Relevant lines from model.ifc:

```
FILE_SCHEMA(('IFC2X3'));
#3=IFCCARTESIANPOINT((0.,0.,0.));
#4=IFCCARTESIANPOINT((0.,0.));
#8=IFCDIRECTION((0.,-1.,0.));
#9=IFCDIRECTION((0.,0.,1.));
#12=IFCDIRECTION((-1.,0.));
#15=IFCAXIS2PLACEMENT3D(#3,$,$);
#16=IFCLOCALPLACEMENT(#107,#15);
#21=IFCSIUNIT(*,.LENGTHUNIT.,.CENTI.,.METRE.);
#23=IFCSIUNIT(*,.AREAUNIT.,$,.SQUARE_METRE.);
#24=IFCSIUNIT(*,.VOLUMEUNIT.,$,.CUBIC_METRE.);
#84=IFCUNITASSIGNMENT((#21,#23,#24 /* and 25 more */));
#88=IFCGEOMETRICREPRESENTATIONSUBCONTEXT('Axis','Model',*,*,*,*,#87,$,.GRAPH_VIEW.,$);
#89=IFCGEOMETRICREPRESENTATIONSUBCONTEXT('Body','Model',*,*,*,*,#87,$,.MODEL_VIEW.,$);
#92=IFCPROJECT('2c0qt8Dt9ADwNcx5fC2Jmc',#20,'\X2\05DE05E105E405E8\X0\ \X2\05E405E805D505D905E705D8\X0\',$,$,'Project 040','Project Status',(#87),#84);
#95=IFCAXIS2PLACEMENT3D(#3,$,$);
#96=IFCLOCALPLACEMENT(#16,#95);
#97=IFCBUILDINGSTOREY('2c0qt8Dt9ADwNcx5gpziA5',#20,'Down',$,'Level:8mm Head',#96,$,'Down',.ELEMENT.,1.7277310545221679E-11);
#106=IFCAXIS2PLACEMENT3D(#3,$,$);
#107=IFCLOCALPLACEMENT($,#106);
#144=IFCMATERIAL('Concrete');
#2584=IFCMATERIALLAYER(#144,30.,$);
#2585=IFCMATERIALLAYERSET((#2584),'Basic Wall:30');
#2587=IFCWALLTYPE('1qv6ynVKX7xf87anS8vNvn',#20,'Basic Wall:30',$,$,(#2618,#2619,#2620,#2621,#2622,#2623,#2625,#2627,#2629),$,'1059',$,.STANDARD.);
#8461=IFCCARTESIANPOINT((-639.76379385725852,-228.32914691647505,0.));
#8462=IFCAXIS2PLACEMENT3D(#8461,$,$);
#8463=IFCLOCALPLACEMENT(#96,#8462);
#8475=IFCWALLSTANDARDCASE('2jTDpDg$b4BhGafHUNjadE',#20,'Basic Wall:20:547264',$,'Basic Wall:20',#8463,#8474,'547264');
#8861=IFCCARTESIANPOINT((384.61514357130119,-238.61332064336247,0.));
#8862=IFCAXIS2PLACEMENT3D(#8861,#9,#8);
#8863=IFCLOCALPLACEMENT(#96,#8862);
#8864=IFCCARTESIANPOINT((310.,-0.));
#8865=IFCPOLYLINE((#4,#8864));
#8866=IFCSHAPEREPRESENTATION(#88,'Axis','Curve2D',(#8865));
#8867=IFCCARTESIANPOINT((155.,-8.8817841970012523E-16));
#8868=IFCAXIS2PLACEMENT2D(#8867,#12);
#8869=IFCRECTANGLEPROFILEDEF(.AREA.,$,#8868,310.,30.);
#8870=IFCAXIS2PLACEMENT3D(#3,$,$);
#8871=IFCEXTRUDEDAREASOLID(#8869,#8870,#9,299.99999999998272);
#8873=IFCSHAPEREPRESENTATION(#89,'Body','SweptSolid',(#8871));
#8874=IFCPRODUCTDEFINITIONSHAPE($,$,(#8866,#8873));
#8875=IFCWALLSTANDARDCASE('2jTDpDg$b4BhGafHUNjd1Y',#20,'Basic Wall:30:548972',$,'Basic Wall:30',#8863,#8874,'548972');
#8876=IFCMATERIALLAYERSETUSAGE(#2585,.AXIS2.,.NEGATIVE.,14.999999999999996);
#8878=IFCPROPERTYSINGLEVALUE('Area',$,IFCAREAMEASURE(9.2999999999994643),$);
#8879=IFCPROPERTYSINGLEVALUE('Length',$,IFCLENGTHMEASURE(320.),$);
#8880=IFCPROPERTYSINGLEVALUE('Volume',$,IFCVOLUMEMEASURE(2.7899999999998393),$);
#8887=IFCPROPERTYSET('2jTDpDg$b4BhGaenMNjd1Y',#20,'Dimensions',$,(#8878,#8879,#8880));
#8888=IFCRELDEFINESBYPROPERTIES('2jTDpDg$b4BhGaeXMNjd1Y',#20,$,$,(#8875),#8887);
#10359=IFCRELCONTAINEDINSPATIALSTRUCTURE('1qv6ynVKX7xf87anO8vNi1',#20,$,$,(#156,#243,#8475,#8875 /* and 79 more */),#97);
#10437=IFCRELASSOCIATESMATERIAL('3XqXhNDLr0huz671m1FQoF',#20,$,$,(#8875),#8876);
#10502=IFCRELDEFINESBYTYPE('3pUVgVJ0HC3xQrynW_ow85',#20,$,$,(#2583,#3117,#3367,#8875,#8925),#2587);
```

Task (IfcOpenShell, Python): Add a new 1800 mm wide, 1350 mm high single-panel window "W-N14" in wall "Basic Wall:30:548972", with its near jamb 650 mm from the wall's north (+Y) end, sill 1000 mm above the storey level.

```python
import numpy as np
import ifcopenshell
import ifcopenshell.api.feature
import ifcopenshell.api.geometry
import ifcopenshell.api.pset
import ifcopenshell.api.root
import ifcopenshell.api.spatial
import ifcopenshell.api.type
import ifcopenshell.geom
import ifcopenshell.util.element
import ifcopenshell.util.placement
import ifcopenshell.util.representation
import ifcopenshell.util.shape
import ifcopenshell.util.unit

model = ifcopenshell.open("model.ifc")
unit_scale = ifcopenshell.util.unit.calculate_unit_scale(model)
area_scale = ifcopenshell.util.unit.calculate_unit_scale(model, "AREAUNIT")
volume_scale = ifcopenshell.util.unit.calculate_unit_scale(model, "VOLUMEUNIT")
settings = ifcopenshell.geom.settings()


def volume(element):
    """Net volume in cubic metres, openings subtracted."""
    shape = ifcopenshell.geom.create_shape(settings, element)
    return ifcopenshell.util.shape.get_volume(shape.geometry)


wall = model.by_guid("2jTDpDg$b4BhGafHUNjd1Y")
storey = ifcopenshell.util.element.get_container(wall, ifc_class="IfcBuildingStorey")
context = ifcopenshell.util.representation.get_context(model, "Model", "Body", "MODEL_VIEW")
before = volume(wall)

width, height, from_end, sill = 1.8, 1.35, 0.65, 1  # metres

# The wall runs along its own X axis, and the end named is its -X end.
wall_shape = ifcopenshell.geom.create_shape(settings, wall)
x, y, z = ifcopenshell.util.shape.get_vertices(wall_shape.geometry).T
start = x.min() + from_end
face, thickness = float(y.min()), float(y.max() - y.min())
wall_matrix = ifcopenshell.util.placement.get_local_placement(wall.ObjectPlacement)
level = ifcopenshell.util.placement.get_local_placement(storey.ObjectPlacement)[2, 3]


def in_wall(x, y):
    """Placement at x, y metres in the wall's axes, at sill height."""
    matrix = wall_matrix.copy()
    matrix[:, 3] = wall_matrix @ np.array([x / unit_scale, y / unit_scale, 0.0, 1.0])
    matrix[2, 3] = level + sill / unit_scale
    return matrix


# Opening: a box that overshoots both wall faces by 50 mm.
opening = ifcopenshell.api.root.create_entity(model, ifc_class="IfcOpeningElement")
box = ifcopenshell.api.geometry.add_wall_representation(
    model, context=context, length=width, height=height, thickness=thickness + 0.1
)
ifcopenshell.api.geometry.assign_representation(model, product=opening, representation=box)
ifcopenshell.api.geometry.edit_object_placement(model, product=opening, matrix=in_wall(start, face - 0.05), is_si=False)
ifcopenshell.api.feature.add_feature(model, feature=opening, element=wall)

window = ifcopenshell.api.root.create_entity(model, ifc_class="IfcWindow", name="W-N14")
window.OverallWidth, window.OverallHeight = width / unit_scale, height / unit_scale
body = ifcopenshell.api.geometry.add_window_representation(
    model,
    context=context,
    overall_width=window.OverallWidth,
    overall_height=window.OverallHeight,
    partition_type="SINGLE_PANEL",
)
ifcopenshell.api.geometry.assign_representation(model, product=window, representation=body)
ifcopenshell.api.spatial.assign_container(model, products=[window], relating_structure=storey)
fills = ifcopenshell.api.feature.add_filling(model, opening=opening, element=window)
fills.OwnerHistory = window.OwnerHistory  # required in IFC2X3

# IFC2X3 keeps the operation on the window style.
style = ifcopenshell.api.root.create_entity(model, ifc_class="IfcWindowStyle", name="W-N14")
style.OperationType, style.ConstructionType = "SINGLE_PANEL", "NOTDEFINED"
style.ParameterTakesPrecedence = style.Sizeable = False
ifcopenshell.api.type.assign_type(model, related_objects=[window], relating_type=style)

# Centre the window in the wall's thickness.
ifcopenshell.api.geometry.edit_object_placement(model, product=window, matrix=in_wall(start, face), is_si=False)
window_shape = ifcopenshell.geom.create_shape(settings, window)
depth = ifcopenshell.util.shape.get_vertices(window_shape.geometry)[:, 1]
offset = face + thickness / 2 - (depth.min() + depth.max()) / 2
ifcopenshell.api.geometry.edit_object_placement(model, product=window, matrix=in_wall(start, offset), is_si=False)

after = volume(wall)

# Update the wall's stored quantities.
pset = model.by_id(ifcopenshell.util.element.get_pset(wall, "Dimensions", should_inherit=False)["id"])
ifcopenshell.api.pset.edit_pset(model, pset=pset, properties={
    "Area": model.create_entity("IfcAreaMeasure", after / thickness / area_scale),
    "Volume": model.create_entity("IfcVolumeMeasure", after / volume_scale),
})

print(f"wall volume {before:.3f} -> {after:.3f} m3")

model.write("model_updated.ifc")
```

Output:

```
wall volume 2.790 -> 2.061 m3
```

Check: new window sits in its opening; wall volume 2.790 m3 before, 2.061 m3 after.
